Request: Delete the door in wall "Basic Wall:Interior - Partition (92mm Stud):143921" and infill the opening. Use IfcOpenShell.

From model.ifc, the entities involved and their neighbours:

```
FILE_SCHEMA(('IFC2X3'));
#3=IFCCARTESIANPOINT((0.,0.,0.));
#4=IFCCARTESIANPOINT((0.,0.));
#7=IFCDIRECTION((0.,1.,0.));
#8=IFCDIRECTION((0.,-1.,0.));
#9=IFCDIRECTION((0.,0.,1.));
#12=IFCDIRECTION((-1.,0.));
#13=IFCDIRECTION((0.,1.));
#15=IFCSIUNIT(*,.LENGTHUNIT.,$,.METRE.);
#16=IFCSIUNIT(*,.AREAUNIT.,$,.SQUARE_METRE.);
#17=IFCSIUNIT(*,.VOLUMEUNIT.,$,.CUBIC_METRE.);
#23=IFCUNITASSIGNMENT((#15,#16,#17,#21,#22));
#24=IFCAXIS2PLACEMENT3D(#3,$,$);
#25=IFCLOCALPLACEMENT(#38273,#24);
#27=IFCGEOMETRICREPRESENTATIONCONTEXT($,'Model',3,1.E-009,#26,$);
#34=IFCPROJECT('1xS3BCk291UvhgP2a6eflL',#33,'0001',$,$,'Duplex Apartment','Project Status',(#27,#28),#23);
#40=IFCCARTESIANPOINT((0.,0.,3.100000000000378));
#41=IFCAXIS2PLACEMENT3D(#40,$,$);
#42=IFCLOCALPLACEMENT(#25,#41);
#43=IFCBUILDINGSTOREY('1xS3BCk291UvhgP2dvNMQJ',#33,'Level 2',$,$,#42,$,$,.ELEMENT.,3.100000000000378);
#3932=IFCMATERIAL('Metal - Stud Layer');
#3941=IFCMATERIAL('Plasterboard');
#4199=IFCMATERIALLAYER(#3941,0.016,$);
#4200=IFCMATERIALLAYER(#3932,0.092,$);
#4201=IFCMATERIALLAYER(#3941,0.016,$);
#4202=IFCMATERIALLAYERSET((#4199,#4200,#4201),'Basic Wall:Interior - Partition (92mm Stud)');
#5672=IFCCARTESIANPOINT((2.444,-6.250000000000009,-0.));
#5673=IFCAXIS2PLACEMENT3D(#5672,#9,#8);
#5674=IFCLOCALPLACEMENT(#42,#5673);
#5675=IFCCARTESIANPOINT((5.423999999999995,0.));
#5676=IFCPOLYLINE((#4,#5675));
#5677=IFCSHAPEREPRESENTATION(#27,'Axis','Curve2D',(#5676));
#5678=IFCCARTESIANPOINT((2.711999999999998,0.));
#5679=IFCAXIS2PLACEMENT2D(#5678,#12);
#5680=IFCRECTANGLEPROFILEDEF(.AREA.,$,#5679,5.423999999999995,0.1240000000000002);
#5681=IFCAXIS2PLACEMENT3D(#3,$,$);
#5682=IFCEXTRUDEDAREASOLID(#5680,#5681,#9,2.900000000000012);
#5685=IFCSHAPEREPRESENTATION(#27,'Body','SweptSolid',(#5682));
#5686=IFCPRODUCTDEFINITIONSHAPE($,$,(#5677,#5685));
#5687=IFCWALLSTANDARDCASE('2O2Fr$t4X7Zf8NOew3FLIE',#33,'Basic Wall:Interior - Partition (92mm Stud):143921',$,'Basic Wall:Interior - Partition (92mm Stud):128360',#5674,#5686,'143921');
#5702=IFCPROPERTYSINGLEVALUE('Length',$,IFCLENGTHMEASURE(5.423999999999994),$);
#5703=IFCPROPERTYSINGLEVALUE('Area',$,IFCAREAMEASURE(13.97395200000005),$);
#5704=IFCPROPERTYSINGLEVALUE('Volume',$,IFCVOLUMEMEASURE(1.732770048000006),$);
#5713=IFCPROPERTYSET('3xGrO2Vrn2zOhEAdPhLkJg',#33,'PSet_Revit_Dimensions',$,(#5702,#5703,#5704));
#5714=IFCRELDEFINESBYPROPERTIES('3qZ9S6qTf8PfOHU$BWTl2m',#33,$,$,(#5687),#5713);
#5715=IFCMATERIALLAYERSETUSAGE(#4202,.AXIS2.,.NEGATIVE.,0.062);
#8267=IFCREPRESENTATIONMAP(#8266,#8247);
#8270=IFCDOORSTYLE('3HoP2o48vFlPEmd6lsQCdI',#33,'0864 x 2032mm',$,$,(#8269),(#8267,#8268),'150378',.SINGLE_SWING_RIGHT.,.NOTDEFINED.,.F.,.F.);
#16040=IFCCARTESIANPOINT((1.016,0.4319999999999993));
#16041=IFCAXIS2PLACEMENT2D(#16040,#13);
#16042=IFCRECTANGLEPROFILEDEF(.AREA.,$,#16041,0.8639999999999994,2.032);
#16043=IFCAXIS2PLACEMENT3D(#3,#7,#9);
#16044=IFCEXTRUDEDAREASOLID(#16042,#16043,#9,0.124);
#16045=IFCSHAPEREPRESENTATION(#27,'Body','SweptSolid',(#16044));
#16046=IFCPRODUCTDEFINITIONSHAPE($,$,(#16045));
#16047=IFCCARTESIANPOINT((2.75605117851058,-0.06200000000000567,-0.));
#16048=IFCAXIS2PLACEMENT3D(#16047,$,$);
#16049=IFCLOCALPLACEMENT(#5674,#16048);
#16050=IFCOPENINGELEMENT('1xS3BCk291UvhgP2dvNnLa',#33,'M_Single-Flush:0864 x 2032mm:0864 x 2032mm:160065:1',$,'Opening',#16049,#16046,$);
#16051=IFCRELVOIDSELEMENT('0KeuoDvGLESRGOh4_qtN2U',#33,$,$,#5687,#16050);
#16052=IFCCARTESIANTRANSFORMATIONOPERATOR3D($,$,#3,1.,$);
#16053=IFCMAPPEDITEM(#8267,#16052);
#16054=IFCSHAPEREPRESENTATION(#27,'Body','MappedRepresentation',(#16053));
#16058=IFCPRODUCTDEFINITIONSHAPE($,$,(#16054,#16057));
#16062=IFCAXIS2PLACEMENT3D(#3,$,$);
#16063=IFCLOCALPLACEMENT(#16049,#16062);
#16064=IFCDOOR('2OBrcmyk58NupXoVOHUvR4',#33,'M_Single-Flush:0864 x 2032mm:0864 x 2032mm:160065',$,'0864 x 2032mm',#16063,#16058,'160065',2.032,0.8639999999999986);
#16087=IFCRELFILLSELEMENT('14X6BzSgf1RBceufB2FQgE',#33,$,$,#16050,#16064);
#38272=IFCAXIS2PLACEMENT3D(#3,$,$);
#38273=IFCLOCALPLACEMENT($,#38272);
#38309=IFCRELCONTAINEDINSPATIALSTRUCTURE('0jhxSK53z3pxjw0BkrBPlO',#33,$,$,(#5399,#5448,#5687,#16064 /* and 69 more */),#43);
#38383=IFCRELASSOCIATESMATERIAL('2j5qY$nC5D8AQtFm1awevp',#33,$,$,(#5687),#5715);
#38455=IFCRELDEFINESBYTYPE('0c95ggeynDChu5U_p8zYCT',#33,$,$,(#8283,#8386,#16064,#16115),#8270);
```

```python
import ifcopenshell
import ifcopenshell.api.feature
import ifcopenshell.api.pset
import ifcopenshell.api.root
import ifcopenshell.geom
import ifcopenshell.util.element
import ifcopenshell.util.shape
import ifcopenshell.util.unit

model = ifcopenshell.open("model.ifc")
area_scale = ifcopenshell.util.unit.calculate_unit_scale(model, "AREAUNIT")
volume_scale = ifcopenshell.util.unit.calculate_unit_scale(model, "VOLUMEUNIT")
settings = ifcopenshell.geom.settings()


def volume(element):
    """Net volume in cubic metres, openings subtracted."""
    shape = ifcopenshell.geom.create_shape(settings, element)
    return ifcopenshell.util.shape.get_volume(shape.geometry)


door = model.by_guid("2OBrcmyk58NupXoVOHUvR4")
opening = door.FillsVoids[0].RelatingOpeningElement
wall = opening.VoidsElements[0].RelatingBuildingElement
before = volume(wall)

ifcopenshell.api.root.remove_product(model, product=door)
ifcopenshell.api.feature.remove_feature(model, feature=opening)

after = volume(wall)
thickness = 0.124  # wall thickness in metres

# Update the wall's stored quantities.
pset = model.by_id(ifcopenshell.util.element.get_pset(wall, "PSet_Revit_Dimensions", should_inherit=False)["id"])
ifcopenshell.api.pset.edit_pset(model, pset=pset, properties={
    "Area": model.create_entity("IfcAreaMeasure", after / thickness / area_scale),
    "Volume": model.create_entity("IfcVolumeMeasure", after / volume_scale),
})

print(f"wall volume {before:.3f} -> {after:.3f} m3")

model.write("model_updated.ifc")
```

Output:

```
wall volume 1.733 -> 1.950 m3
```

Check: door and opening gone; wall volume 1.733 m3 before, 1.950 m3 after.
